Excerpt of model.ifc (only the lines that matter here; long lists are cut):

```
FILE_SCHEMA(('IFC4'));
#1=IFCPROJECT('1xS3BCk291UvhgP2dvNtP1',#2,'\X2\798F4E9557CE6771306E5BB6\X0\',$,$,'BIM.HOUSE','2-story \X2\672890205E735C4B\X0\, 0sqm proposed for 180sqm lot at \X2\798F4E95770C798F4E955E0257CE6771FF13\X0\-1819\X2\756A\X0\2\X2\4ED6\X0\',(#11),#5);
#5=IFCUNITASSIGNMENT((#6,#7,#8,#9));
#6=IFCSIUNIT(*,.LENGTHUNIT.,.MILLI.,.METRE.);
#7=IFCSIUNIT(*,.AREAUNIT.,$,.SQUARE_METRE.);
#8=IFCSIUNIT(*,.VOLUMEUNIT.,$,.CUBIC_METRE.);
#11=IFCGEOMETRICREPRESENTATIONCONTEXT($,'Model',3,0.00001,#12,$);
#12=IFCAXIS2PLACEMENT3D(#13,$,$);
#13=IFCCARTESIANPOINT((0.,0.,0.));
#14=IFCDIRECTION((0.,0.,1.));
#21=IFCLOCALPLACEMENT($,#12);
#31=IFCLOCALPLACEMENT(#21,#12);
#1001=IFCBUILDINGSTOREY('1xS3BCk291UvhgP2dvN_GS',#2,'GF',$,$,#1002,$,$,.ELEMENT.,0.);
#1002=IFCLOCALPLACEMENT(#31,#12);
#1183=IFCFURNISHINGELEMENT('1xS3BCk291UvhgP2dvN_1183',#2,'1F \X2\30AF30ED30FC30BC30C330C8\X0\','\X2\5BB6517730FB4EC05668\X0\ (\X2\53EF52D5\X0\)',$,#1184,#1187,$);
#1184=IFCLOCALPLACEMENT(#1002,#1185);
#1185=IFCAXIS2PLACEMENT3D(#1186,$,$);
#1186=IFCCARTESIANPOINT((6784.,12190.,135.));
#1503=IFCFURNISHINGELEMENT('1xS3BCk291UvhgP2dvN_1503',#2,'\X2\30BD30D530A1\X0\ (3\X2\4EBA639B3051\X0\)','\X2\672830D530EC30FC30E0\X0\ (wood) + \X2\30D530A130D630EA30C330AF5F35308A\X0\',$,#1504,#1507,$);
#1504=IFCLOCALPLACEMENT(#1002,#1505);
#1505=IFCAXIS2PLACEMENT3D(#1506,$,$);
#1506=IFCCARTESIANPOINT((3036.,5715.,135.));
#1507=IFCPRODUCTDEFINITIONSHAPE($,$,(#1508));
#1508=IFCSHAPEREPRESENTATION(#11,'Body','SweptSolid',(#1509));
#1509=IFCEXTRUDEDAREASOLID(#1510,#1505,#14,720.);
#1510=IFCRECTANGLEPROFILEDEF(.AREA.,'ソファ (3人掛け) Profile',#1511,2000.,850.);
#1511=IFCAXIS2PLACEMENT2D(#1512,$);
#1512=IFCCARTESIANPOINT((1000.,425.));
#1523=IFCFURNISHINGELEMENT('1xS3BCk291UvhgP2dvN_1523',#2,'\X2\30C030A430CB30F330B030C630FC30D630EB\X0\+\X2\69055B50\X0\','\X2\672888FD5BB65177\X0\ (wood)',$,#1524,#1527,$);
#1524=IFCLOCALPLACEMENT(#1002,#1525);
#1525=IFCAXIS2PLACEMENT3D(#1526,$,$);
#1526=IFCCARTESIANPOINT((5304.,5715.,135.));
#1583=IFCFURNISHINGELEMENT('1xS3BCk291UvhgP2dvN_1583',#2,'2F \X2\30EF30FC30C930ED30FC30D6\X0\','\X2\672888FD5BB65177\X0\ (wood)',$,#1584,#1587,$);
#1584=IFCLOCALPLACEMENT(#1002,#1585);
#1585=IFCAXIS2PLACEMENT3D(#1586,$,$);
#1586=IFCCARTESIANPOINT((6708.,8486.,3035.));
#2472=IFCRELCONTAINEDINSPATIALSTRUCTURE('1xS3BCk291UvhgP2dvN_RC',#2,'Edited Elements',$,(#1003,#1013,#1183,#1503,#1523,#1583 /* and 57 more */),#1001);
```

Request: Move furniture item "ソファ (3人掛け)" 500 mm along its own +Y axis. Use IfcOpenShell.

```python
import ifcopenshell
import ifcopenshell.api.geometry
import ifcopenshell.util.placement

model = ifcopenshell.open("model.ifc")

item = model.by_id(1503)
matrix = ifcopenshell.util.placement.get_local_placement(item.ObjectPlacement)
matrix[:3, 3] += matrix[:3, 1] * 500.0
ifcopenshell.api.geometry.edit_object_placement(model, product=item, matrix=matrix, is_si=False)

print(ifcopenshell.util.placement.get_local_placement(item.ObjectPlacement).round(3) + 0.0)

model.write("model_v2.ifc")
```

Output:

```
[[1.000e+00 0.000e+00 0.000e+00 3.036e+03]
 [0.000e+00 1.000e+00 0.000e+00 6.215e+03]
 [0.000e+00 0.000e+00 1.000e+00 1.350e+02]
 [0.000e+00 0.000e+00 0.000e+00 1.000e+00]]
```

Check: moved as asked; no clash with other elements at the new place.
